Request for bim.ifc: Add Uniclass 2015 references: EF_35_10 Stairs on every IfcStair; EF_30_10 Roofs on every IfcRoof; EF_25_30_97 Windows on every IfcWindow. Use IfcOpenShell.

First a look at what the model holds.

```python
import ifcopenshell

model = ifcopenshell.open("bim.ifc")
print(model.schema)
print("classifications:", [c.Name for c in model.by_type("IfcClassification")])
for ifc_class in ("IfcDoor", "IfcRoof", "IfcStair", "IfcWall", "IfcWindow"):
    print(ifc_class, len(model.by_type(ifc_class)))
```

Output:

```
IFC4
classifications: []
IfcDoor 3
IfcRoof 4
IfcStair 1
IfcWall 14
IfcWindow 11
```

```python
import ifcopenshell
import ifcopenshell.api.classification

model = ifcopenshell.open("bim.ifc")

system = ifcopenshell.api.classification.add_classification(model, classification="Uniclass 2015")

codes = {
    "IfcStair": ("EF_35_10", "Stairs"),
    "IfcRoof": ("EF_30_10", "Roofs"),
    "IfcWindow": ("EF_25_30_97", "Windows"),
}
for ifc_class, (code, name) in codes.items():
    products = model.by_type(ifc_class)
    ifcopenshell.api.classification.add_reference(
        model, products=products, classification=system, identification=code, name=name
    )
    print(code, len(products))

model.write("bim_updated.ifc")
```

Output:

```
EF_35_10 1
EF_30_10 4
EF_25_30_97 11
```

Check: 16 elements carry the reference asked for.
